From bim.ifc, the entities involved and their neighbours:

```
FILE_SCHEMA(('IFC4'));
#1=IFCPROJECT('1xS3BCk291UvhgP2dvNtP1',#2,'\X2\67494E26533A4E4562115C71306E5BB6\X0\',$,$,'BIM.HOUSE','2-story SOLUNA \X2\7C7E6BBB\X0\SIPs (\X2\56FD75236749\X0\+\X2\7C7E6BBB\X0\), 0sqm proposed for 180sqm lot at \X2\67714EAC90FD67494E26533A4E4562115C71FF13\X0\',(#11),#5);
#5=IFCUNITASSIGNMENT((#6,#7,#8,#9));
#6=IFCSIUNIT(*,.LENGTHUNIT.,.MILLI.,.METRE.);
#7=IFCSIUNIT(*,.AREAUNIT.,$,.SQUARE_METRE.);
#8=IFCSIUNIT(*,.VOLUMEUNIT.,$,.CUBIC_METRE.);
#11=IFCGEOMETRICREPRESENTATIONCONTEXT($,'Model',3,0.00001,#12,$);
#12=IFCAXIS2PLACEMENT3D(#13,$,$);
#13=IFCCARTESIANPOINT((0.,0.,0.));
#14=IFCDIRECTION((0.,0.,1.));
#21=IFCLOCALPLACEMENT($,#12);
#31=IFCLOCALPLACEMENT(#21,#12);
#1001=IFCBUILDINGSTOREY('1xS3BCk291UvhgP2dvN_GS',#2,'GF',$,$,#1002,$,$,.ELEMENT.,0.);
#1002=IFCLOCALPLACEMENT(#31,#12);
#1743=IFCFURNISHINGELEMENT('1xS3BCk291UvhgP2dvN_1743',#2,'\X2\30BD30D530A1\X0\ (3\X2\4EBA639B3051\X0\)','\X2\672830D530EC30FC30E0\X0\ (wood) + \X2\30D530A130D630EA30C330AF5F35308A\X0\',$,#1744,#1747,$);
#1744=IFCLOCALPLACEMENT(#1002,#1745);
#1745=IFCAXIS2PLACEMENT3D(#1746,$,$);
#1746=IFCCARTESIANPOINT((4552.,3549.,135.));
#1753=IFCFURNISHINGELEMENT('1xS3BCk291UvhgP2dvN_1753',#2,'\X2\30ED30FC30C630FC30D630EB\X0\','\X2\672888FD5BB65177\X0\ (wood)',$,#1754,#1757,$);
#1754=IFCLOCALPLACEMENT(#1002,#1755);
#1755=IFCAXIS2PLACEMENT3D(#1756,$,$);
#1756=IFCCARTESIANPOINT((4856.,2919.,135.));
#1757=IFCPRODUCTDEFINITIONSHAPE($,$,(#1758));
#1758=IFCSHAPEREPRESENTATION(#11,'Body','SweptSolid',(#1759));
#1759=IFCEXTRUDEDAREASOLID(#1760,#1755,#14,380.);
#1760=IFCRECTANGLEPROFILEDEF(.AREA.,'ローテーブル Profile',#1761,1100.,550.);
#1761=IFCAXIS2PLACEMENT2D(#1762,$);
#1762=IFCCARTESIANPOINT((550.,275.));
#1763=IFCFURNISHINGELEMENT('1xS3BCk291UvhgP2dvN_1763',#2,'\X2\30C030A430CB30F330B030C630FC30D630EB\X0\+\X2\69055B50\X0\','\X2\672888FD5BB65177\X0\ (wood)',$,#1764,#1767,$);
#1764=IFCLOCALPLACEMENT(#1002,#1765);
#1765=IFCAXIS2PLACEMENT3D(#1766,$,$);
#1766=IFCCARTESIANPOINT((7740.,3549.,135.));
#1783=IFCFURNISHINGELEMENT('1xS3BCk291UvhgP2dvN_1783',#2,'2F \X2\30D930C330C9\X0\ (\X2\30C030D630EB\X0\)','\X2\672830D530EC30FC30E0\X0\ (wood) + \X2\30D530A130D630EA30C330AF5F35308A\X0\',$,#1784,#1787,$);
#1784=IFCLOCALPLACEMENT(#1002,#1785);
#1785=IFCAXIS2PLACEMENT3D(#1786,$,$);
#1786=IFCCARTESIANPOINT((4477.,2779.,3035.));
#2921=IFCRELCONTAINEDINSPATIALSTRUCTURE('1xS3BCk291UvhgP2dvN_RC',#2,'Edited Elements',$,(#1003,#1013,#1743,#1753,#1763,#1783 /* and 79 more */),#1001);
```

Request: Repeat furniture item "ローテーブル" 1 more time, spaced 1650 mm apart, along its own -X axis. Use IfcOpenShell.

```python
import ifcopenshell
import ifcopenshell.api.geometry
import ifcopenshell.api.root
import ifcopenshell.util.element
import ifcopenshell.util.placement
import ifcopenshell.util.unit

model = ifcopenshell.open("bim.ifc")
unit_scale = ifcopenshell.util.unit.calculate_unit_scale(model)


def reuse_history(source, copy):
    """copy_class also copies each property set's owner history, people and application; keep the originals."""
    for rel in copy.IsDefinedBy:
        if rel.is_a("IfcRelDefinesByProperties") and (history := rel.RelatingPropertyDefinition.OwnerHistory):
            rel.RelatingPropertyDefinition.OwnerHistory = source.OwnerHistory
            ifcopenshell.util.element.remove_deep2(model, history)


source = model.by_guid("1xS3BCk291UvhgP2dvN_1753")
base = ifcopenshell.util.placement.get_local_placement(source.ObjectPlacement)
step = -base[:3, 0] * 1.65 / unit_scale

for i in range(1, 2):
    copy = ifcopenshell.api.root.copy_class(model, product=source)
    copy.Representation = ifcopenshell.util.element.copy_deep(
        model, source.Representation, exclude=["IfcGeometricRepresentationContext", "IfcRepresentationMap"]
    )
    reuse_history(source, copy)
    matrix = base.copy()
    matrix[:3, 3] += i * step
    print("added at", matrix[:3, 3].round(3) + 0.0)
    ifcopenshell.api.geometry.edit_object_placement(model, product=copy, matrix=matrix, is_si=False)

model.write("bim_rev.ifc")
```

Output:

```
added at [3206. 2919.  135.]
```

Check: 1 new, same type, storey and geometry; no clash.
